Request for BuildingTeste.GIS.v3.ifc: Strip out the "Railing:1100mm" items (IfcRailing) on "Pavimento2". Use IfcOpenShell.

First a look at what the model holds.

```python
import ifcopenshell
import ifcopenshell.util.element

model = ifcopenshell.open("BuildingTeste.GIS.v3.ifc")
print(model.schema)
storey = next(s for s in model.by_type("IfcBuildingStorey") if s.Name == "Pavimento2")
railings = [e for e in ifcopenshell.util.element.get_decomposition(storey) if e.is_a("IfcRailing")]
seen = {}
for e in railings:
    element_type = ifcopenshell.util.element.get_type(e)
    name = element_type.Name if element_type not in (None, e) else None
    seen[name] = seen.get(name, 0) + 1
for name, count in sorted(seen.items(), key=str):
    print(count, "x", name)
```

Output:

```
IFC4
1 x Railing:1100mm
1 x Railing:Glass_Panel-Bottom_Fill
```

```python
import ifcopenshell
import ifcopenshell.api.root
import ifcopenshell.util.element

model = ifcopenshell.open("BuildingTeste.GIS.v3.ifc")

storey = next(s for s in model.by_type("IfcBuildingStorey") if s.Name == "Pavimento2")
railings = [e for e in ifcopenshell.util.element.get_decomposition(storey) if e.is_a("IfcRailing")]
targets = [e for e in railings if (t := ifcopenshell.util.element.get_type(e)) not in (None, e) and t.Name == "Railing:1100mm"]

for e in targets:
    ifcopenshell.api.root.remove_product(model, product=e)
print(len(targets), "removed")

model.write("BuildingTeste.GIS.v3_v2.ifc")
```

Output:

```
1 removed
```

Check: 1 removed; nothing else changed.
